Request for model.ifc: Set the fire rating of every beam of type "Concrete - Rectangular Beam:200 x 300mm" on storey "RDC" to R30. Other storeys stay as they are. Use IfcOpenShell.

First a look at what the model holds.

```python
import ifcopenshell
import ifcopenshell.util.element

model = ifcopenshell.open("model.ifc")
print(model.schema)
storey = next(s for s in model.by_type("IfcBuildingStorey") if s.Name == "RDC")
beams = [e for e in ifcopenshell.util.element.get_decomposition(storey) if e.is_a("IfcBeam")]
seen = {}
for e in beams:
    element_type = ifcopenshell.util.element.get_type(e)
    key = (element_type.Name if element_type != e and element_type else None, ifcopenshell.util.element.get_pset(e, "Pset_BeamCommon", "FireRating"))
    seen[key] = seen.get(key, 0) + 1
for (name, value), count in sorted(seen.items(), key=str):
    print(count, "x", name, "|", value)
```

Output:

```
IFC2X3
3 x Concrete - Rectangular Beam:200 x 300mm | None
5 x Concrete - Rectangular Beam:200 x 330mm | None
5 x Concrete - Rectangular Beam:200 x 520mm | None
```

```python
import ifcopenshell
import ifcopenshell.api.pset
import ifcopenshell.util.element

model = ifcopenshell.open("model.ifc")

storey = next(s for s in model.by_type("IfcBuildingStorey") if s.Name == "RDC")
beams = [e for e in ifcopenshell.util.element.get_decomposition(storey) if e.is_a("IfcBeam")]

count = 0
for e in beams:
    element_type = ifcopenshell.util.element.get_type(e)
    if element_type in (None, e) or element_type.Name != "Concrete - Rectangular Beam:200 x 300mm":
        continue
    # add_pset returns the element's existing set when there is one.
    pset = ifcopenshell.api.pset.add_pset(model, product=e, name="Pset_BeamCommon")
    ifcopenshell.api.pset.edit_pset(model, pset=pset, properties={"FireRating": "R30"})
    count += 1

print(count, "beams updated")

model.write("model_updated.ifc")
```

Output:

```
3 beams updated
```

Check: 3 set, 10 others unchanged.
